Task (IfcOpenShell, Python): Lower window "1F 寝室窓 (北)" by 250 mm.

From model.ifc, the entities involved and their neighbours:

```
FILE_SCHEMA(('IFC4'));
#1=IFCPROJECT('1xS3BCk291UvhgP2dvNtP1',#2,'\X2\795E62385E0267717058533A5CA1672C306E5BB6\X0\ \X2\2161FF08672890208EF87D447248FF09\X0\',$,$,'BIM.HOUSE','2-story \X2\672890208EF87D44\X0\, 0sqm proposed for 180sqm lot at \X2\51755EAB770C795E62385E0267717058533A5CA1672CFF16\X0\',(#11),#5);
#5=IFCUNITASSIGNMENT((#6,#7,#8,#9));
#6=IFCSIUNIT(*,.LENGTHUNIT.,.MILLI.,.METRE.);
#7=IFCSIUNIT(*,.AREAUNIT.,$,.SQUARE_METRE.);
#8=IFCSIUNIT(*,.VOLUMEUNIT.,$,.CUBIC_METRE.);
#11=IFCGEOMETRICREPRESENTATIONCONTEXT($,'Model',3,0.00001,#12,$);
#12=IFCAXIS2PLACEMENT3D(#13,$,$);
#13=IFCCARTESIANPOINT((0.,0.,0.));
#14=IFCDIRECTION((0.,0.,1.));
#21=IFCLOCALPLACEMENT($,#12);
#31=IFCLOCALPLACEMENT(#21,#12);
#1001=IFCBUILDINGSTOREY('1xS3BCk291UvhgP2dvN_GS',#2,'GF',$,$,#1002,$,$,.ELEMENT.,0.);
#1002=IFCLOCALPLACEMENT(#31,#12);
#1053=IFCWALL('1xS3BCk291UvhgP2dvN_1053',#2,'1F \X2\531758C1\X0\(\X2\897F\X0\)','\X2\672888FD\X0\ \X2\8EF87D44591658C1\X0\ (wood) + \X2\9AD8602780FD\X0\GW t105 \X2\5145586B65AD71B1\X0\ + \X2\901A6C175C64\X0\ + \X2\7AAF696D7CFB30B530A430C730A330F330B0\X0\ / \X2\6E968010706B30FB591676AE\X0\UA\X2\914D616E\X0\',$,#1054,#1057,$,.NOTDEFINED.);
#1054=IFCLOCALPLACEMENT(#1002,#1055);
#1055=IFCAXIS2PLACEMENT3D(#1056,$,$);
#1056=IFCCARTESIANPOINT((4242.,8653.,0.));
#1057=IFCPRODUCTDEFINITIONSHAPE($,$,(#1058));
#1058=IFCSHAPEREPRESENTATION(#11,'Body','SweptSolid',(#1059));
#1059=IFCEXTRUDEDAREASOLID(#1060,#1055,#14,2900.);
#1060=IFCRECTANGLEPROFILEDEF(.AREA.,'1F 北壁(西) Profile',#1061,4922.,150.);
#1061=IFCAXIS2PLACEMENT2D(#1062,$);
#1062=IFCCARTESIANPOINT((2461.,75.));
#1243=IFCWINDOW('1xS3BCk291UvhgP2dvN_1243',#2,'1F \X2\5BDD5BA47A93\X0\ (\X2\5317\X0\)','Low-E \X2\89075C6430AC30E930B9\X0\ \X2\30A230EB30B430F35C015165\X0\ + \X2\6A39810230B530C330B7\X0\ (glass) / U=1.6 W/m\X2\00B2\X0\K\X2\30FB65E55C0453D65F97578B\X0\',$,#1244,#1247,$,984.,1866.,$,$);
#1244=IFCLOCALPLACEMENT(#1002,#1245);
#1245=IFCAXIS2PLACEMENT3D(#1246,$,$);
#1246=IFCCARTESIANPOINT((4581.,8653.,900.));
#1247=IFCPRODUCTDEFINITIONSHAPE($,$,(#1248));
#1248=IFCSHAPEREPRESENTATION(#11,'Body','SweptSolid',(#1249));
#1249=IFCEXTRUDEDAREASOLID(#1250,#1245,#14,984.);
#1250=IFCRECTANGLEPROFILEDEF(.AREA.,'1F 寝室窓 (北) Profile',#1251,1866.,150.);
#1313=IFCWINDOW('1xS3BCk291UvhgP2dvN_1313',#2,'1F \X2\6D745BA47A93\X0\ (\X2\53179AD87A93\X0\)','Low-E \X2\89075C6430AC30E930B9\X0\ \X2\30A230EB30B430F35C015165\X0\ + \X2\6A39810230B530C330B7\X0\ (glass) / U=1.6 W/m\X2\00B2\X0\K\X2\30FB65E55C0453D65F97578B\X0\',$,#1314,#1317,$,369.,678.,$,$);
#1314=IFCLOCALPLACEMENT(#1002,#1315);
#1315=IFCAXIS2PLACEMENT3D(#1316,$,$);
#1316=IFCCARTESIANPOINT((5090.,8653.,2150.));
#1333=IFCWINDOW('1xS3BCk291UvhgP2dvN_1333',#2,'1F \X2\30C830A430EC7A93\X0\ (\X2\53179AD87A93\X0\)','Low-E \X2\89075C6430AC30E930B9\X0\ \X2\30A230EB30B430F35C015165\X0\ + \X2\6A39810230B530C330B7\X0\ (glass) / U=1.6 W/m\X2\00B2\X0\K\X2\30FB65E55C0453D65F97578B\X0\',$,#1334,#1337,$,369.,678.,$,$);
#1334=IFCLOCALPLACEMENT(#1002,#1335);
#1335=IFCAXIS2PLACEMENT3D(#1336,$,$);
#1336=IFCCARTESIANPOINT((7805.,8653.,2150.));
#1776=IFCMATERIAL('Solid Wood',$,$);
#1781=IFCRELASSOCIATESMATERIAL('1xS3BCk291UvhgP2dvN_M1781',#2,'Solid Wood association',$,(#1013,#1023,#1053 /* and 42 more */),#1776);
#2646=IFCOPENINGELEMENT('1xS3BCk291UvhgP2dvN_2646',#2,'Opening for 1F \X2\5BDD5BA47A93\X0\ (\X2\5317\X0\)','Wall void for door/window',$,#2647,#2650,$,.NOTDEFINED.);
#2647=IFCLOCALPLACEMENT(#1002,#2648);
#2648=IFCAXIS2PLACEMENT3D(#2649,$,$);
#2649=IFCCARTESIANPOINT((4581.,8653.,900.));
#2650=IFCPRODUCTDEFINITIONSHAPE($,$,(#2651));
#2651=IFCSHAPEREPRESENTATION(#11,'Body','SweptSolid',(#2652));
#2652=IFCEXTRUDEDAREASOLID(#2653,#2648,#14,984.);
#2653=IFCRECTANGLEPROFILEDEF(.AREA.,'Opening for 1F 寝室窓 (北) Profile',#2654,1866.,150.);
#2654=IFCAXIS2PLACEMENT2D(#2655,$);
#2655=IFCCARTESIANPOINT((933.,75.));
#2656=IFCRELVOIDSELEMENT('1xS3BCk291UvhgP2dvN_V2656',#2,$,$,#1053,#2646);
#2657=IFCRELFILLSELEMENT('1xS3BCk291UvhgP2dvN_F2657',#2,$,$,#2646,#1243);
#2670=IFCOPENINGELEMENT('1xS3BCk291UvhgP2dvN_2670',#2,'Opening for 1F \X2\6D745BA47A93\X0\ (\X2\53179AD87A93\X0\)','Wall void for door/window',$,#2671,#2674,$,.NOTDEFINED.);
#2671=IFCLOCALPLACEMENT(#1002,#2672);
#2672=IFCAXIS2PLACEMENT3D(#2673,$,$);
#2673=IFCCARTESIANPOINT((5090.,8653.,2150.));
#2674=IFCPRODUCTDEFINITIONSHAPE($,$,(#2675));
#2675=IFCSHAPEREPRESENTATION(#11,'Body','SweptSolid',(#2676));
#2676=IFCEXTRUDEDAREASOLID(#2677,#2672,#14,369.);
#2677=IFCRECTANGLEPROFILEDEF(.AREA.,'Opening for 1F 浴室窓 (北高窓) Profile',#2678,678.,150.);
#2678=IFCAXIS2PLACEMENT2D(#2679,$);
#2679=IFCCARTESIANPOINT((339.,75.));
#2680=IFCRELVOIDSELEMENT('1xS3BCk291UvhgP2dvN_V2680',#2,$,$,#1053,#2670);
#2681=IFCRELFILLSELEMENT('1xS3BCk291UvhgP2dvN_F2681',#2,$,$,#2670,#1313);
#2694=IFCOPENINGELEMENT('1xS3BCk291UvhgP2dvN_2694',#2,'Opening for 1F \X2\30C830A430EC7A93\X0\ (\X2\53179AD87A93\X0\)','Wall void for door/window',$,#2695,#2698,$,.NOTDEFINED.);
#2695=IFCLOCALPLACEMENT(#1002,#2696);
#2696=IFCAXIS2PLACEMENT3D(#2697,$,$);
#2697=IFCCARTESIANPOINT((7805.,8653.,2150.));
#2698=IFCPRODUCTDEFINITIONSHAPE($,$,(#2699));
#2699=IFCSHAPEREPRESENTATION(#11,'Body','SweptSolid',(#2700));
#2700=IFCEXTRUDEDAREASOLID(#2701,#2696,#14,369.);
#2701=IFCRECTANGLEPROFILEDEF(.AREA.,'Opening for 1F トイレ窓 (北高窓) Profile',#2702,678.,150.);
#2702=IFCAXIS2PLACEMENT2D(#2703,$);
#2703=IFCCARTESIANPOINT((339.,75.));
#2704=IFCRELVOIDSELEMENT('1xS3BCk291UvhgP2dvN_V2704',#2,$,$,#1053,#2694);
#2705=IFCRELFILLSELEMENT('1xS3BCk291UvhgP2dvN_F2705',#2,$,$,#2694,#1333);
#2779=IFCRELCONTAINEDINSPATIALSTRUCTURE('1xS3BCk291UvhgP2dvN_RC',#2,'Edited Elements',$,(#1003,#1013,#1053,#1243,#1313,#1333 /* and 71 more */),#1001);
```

```python
import numpy as np
import ifcopenshell
import ifcopenshell.api.geometry
import ifcopenshell.util.placement
import ifcopenshell.util.unit

model = ifcopenshell.open("model.ifc")
unit_scale = ifcopenshell.util.unit.calculate_unit_scale(model)

window = model.by_id(1243)
opening = window.FillsVoids[0].RelatingOpeningElement
dz = -0.25 / unit_scale

shift = np.array([0.0, 0.0, dz])
# The window is not placed relative to its opening, so move both.
for product in (opening, window):
    matrix = ifcopenshell.util.placement.get_local_placement(product.ObjectPlacement)
    matrix[:3, 3] += shift
    ifcopenshell.api.geometry.edit_object_placement(model, product=product, matrix=matrix, is_si=False)

print(f"moved by {dz * unit_scale:+.3f} m")

model.write("model_updated.ifc")
```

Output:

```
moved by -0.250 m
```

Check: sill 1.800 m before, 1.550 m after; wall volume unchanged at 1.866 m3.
